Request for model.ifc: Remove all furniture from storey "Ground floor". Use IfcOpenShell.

First a look at what the model holds.

```python
import ifcopenshell
import ifcopenshell.util.element

model = ifcopenshell.open("model.ifc")
print(model.schema)
storey = next(s for s in model.by_type("IfcBuildingStorey") if s.Name == "Ground floor")
furniture = [e for e in ifcopenshell.util.element.get_decomposition(storey) if e.is_a("IfcFurnishingElement")]
seen = {}
for e in furniture:
    element_type = ifcopenshell.util.element.get_type(e)
    name = element_type.Name if element_type not in (None, e) else None
    seen[name] = seen.get(name, 0) + 1
for name, count in sorted(seen.items(), key=str):
    print(count, "x", name)
```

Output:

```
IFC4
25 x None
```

```python
import ifcopenshell
import ifcopenshell.api.root
import ifcopenshell.util.element

model = ifcopenshell.open("model.ifc")

storey = next(s for s in model.by_type("IfcBuildingStorey") if s.Name == "Ground floor")
furniture = [e for e in ifcopenshell.util.element.get_decomposition(storey) if e.is_a("IfcFurnishingElement")]

for e in furniture:
    ifcopenshell.api.root.remove_product(model, product=e)
print(len(furniture), "removed")

model.write("model_updated.ifc")
```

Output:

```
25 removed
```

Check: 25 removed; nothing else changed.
